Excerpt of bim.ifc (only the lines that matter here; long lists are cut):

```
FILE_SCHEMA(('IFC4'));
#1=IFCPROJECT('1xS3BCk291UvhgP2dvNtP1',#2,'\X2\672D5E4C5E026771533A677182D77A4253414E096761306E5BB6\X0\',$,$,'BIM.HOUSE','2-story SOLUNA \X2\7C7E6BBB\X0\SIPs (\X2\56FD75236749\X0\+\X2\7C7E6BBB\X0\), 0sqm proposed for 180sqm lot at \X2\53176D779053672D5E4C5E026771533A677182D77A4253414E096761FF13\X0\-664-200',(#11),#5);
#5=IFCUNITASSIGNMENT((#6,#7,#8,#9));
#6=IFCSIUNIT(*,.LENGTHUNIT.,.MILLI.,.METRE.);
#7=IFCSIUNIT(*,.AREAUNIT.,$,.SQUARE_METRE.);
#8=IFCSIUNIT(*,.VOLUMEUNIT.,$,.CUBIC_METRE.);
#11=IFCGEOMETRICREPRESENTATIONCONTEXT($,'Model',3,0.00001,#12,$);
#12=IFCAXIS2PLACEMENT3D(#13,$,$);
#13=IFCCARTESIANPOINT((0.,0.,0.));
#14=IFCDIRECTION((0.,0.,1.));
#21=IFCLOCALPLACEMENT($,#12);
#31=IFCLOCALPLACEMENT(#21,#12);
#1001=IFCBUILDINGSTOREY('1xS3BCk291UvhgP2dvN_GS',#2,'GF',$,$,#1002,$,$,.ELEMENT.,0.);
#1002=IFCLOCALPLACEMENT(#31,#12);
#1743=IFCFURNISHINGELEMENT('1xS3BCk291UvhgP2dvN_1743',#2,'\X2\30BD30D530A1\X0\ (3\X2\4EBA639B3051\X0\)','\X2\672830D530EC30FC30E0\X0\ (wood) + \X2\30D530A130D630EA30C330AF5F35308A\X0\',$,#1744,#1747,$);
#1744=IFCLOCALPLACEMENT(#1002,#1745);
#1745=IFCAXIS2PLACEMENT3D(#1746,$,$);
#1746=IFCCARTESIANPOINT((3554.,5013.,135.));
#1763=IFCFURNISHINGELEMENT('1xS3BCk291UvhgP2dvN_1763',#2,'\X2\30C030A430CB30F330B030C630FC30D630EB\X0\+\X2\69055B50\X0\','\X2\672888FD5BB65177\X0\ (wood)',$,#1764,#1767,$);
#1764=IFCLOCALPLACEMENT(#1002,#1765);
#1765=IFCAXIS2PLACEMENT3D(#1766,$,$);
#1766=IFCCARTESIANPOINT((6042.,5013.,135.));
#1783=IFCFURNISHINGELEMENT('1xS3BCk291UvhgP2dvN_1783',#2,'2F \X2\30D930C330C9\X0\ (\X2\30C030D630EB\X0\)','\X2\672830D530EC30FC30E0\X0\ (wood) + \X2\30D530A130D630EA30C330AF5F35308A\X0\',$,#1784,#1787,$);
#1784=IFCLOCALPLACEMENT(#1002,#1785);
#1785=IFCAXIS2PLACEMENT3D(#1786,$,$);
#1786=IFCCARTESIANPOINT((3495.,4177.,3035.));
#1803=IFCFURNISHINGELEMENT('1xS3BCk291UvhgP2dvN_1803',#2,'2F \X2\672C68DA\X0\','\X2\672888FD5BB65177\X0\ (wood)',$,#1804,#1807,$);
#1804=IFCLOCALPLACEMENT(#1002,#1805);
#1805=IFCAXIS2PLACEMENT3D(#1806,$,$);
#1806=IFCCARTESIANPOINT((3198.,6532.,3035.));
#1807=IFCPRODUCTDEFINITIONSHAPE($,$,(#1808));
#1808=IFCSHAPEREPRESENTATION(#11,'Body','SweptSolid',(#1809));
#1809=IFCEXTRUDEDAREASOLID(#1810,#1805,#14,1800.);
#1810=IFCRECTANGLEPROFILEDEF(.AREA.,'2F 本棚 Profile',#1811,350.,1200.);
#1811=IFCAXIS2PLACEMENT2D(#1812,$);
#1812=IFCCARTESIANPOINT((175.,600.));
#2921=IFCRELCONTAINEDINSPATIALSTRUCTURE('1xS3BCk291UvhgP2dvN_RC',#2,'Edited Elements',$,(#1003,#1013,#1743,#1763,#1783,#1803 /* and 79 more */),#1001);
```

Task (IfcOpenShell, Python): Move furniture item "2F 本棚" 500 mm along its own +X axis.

```python
import ifcopenshell
import ifcopenshell.api.geometry
import ifcopenshell.util.placement
import ifcopenshell.util.unit

model = ifcopenshell.open("bim.ifc")
unit_scale = ifcopenshell.util.unit.calculate_unit_scale(model)

item = model.by_guid("1xS3BCk291UvhgP2dvN_1803")
matrix = ifcopenshell.util.placement.get_local_placement(item.ObjectPlacement)
matrix[:3, 3] += matrix[:3, 0] * 0.5 / unit_scale
ifcopenshell.api.geometry.edit_object_placement(model, product=item, matrix=matrix, is_si=False)

print(ifcopenshell.util.placement.get_local_placement(item.ObjectPlacement).round(3) + 0.0)

model.write("bim_v2.ifc")
```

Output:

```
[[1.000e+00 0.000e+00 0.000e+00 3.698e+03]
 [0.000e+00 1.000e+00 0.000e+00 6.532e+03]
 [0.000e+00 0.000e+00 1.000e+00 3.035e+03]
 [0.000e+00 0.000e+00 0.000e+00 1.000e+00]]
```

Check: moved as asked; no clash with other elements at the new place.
